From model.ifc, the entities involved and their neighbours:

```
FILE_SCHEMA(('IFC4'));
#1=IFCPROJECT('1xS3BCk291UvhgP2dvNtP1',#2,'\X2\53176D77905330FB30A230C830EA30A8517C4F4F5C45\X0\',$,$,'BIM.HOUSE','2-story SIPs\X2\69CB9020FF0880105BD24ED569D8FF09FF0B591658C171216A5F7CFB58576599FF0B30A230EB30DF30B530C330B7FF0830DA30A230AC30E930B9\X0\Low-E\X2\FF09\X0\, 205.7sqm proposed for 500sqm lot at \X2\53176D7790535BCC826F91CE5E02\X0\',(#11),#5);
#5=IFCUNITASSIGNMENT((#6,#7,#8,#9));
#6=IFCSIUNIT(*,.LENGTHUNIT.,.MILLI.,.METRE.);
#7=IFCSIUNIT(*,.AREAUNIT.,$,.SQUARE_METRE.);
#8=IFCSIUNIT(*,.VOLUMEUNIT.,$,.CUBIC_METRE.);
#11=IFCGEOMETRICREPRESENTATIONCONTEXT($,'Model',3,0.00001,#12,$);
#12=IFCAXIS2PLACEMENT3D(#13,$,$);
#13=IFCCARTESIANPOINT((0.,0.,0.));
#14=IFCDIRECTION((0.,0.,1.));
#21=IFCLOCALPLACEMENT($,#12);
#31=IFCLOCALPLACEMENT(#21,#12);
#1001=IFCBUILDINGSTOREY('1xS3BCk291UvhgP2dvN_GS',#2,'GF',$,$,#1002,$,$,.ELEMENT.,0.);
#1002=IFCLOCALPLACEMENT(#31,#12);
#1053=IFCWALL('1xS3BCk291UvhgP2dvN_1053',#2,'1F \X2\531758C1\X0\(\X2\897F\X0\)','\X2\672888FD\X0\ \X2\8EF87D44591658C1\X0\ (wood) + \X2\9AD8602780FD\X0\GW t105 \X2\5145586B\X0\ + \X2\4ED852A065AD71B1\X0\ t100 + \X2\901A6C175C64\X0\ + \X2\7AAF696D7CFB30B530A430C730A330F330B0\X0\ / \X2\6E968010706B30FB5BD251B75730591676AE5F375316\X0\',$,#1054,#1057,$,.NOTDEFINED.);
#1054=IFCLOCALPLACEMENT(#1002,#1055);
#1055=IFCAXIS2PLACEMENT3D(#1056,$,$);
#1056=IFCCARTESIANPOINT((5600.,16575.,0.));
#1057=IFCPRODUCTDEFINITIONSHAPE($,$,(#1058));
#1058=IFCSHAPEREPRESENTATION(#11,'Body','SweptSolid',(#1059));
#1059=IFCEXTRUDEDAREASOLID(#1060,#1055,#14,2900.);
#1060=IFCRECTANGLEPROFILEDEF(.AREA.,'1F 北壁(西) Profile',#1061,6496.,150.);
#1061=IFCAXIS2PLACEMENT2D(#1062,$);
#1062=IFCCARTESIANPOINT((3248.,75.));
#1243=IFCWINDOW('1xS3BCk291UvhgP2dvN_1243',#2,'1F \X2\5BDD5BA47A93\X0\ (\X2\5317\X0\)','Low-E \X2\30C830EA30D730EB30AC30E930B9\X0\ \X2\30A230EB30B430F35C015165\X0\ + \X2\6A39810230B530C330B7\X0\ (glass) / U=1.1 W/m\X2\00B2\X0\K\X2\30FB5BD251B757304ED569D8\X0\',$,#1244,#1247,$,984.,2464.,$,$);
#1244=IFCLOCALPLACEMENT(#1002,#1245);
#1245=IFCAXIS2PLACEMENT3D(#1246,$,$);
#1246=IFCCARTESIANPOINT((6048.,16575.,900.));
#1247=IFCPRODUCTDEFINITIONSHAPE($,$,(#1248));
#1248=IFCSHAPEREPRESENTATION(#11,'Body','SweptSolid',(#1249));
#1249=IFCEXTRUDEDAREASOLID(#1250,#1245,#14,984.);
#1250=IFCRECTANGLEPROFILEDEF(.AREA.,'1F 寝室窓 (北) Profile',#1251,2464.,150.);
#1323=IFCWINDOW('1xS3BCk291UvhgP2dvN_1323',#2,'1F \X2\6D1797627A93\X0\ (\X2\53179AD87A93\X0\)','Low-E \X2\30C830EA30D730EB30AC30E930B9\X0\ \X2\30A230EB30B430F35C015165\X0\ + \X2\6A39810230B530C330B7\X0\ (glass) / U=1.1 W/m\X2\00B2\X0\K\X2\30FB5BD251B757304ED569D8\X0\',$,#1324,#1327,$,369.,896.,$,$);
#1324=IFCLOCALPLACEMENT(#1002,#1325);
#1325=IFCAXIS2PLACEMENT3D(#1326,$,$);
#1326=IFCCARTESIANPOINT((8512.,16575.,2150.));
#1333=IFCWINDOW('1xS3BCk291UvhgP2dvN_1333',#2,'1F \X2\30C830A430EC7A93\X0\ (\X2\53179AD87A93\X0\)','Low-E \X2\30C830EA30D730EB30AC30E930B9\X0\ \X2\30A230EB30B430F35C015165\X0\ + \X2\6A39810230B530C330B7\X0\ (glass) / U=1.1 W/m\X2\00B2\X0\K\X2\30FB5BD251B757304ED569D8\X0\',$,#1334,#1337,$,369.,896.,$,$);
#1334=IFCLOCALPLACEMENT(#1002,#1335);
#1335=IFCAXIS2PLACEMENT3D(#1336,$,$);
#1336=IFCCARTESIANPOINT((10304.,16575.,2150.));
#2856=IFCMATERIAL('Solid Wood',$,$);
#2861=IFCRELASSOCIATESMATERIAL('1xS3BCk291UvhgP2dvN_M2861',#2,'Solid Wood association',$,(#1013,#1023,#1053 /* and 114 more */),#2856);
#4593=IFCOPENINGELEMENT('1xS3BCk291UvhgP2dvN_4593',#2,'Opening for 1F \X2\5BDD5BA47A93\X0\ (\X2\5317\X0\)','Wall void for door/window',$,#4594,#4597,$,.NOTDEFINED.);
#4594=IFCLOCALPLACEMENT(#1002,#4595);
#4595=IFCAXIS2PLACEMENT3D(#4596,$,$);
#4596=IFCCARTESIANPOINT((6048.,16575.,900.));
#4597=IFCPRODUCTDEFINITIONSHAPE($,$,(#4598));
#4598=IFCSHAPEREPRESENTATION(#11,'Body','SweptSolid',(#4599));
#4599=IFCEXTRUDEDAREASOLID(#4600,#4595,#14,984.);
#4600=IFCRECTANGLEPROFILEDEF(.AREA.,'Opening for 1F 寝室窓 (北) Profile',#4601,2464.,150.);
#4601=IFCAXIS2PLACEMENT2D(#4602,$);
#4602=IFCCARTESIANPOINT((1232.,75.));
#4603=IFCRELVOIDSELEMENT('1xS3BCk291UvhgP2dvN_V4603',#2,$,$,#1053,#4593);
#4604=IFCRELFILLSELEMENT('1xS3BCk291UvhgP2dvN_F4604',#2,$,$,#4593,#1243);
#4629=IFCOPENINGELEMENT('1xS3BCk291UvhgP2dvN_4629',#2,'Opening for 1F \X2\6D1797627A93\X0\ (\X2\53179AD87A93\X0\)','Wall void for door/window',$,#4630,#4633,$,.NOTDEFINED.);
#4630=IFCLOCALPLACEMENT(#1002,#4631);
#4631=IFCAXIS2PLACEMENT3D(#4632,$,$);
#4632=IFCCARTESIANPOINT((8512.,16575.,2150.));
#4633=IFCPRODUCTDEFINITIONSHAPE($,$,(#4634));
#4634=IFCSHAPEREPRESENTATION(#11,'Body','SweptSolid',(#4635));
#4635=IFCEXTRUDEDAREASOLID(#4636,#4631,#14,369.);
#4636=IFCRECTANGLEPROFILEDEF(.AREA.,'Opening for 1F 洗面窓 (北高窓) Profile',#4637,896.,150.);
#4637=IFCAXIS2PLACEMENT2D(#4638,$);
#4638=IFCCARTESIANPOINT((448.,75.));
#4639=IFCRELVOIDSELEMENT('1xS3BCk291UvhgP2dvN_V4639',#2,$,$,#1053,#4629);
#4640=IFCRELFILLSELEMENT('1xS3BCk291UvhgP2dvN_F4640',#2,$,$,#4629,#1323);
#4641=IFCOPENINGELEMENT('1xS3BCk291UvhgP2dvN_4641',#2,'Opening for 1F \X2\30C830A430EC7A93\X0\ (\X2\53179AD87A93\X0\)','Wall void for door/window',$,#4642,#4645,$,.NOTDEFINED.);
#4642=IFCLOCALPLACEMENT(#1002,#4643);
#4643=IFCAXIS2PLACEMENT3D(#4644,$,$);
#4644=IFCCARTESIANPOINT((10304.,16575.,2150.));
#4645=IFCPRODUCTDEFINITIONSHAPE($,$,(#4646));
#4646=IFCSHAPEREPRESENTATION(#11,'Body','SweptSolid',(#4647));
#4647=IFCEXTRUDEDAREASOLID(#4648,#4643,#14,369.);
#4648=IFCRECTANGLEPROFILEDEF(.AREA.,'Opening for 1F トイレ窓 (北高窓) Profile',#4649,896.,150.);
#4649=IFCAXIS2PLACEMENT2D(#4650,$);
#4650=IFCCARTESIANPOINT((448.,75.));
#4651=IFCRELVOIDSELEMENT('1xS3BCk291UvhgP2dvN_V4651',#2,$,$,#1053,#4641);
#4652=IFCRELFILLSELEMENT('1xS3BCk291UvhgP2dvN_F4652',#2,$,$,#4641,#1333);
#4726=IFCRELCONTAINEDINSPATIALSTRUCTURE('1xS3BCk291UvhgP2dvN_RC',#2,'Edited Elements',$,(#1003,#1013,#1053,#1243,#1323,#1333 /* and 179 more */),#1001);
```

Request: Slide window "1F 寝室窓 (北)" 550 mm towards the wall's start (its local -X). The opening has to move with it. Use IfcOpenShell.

```python
import ifcopenshell
import ifcopenshell.api.geometry
import ifcopenshell.util.placement

model = ifcopenshell.open("model.ifc")

window = model.by_id(1243)
opening = window.FillsVoids[0].RelatingOpeningElement
wall = opening.VoidsElements[0].RelatingBuildingElement

wall_matrix = ifcopenshell.util.placement.get_local_placement(wall.ObjectPlacement)
shift = wall_matrix[:3, 0] * -550.0
before = ifcopenshell.util.placement.get_local_placement(window.ObjectPlacement)[:3, 3].copy()

# The window is not placed relative to its opening, so move both.
for product in (opening, window):
    matrix = ifcopenshell.util.placement.get_local_placement(product.ObjectPlacement)
    matrix[:3, 3] += shift
    ifcopenshell.api.geometry.edit_object_placement(model, product=product, matrix=matrix, is_si=False)

after = ifcopenshell.util.placement.get_local_placement(window.ObjectPlacement)[:3, 3]
print("window moved by", (after - before).round(3) + 0.0)

model.write("model_updated.ifc")
```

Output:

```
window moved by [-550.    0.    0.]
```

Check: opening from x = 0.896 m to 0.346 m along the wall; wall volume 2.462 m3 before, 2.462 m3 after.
